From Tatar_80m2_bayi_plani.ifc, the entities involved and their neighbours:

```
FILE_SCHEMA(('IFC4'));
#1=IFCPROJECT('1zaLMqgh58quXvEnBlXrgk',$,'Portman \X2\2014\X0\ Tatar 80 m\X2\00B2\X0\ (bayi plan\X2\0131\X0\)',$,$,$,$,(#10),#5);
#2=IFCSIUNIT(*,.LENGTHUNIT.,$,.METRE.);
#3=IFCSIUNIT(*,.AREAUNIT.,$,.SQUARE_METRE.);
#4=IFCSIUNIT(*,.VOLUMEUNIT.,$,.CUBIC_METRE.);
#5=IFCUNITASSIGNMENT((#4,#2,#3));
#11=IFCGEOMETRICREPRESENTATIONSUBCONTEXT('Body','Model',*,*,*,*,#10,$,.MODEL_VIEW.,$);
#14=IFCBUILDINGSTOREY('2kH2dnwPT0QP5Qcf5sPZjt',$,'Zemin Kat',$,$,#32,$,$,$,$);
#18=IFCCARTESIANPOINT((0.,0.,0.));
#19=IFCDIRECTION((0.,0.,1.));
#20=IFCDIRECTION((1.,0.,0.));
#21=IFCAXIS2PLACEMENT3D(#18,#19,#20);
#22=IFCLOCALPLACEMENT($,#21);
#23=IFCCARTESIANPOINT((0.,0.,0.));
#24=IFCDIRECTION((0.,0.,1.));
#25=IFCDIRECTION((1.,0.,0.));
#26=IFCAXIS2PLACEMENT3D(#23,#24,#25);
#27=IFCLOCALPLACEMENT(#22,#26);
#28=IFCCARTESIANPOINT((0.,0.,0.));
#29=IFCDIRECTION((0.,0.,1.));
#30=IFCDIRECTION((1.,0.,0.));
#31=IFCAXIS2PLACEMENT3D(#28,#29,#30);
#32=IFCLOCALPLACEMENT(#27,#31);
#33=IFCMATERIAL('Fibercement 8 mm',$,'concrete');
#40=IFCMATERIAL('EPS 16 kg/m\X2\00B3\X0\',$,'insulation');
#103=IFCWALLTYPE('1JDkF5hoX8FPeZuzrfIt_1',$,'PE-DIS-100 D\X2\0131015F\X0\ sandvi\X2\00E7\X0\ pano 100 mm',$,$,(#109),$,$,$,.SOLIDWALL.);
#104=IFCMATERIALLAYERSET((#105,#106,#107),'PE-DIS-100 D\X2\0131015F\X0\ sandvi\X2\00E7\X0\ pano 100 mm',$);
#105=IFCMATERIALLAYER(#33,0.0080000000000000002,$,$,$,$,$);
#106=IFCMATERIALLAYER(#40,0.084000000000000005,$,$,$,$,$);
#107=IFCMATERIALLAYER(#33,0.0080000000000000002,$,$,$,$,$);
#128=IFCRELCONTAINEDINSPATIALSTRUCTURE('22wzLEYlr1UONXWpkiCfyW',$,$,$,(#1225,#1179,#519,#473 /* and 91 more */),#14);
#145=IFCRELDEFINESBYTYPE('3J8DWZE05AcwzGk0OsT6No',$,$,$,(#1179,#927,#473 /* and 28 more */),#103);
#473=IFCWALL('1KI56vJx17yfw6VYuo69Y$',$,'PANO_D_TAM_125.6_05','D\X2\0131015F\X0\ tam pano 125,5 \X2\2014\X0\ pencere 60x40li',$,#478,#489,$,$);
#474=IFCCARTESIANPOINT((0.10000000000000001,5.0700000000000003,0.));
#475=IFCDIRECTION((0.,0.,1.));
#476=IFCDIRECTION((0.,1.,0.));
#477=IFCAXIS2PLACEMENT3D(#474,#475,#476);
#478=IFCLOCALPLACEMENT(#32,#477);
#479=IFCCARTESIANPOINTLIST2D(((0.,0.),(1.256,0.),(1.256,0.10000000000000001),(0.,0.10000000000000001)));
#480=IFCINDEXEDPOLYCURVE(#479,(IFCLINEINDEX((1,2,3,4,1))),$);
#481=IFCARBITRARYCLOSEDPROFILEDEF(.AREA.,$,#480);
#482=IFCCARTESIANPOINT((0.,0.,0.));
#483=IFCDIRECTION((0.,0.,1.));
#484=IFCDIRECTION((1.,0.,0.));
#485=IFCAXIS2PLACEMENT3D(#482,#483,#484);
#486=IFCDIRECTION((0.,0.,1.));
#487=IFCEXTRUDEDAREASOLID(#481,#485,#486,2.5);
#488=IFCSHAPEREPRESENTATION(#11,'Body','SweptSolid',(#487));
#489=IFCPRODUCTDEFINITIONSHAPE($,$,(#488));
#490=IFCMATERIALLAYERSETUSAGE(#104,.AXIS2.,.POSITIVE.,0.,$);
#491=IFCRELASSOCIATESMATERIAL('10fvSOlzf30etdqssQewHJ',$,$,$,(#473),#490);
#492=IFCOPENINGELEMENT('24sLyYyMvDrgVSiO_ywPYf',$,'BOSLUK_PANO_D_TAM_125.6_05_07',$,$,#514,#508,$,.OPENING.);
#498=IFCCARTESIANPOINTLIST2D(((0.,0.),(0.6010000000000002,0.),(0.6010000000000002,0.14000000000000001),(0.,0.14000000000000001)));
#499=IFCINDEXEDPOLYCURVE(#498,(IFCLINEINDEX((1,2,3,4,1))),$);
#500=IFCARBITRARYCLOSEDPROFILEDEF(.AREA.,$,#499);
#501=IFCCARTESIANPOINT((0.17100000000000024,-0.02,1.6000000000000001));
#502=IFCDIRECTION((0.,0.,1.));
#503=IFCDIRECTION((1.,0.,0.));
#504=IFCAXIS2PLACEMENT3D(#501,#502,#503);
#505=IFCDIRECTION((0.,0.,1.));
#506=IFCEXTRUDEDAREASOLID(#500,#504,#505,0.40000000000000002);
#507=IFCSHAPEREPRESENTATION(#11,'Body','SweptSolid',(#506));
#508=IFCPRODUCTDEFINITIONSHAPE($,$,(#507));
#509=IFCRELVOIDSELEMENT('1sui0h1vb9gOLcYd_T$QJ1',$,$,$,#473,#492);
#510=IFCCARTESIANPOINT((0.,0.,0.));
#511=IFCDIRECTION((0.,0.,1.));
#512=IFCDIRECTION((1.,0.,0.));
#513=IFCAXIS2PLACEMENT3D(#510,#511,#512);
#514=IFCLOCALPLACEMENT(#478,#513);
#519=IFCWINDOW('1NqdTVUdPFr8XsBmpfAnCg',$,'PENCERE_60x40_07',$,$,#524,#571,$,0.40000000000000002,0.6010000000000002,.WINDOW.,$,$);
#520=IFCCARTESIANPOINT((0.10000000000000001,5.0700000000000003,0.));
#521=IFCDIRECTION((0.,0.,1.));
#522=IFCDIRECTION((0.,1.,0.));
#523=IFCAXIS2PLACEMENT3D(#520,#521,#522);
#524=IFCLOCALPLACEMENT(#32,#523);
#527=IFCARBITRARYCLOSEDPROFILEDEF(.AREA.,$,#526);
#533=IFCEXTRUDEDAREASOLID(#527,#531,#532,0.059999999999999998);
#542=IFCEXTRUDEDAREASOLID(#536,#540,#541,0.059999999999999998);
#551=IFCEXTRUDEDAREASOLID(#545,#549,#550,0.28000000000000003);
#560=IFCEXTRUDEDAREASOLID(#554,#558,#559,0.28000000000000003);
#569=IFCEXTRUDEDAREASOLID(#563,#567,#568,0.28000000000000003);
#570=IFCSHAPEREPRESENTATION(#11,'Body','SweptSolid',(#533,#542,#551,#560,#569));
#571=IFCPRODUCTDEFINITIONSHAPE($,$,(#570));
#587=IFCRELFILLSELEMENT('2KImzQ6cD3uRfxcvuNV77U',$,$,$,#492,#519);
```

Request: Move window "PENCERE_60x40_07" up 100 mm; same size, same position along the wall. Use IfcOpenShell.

```python
import numpy as np
import ifcopenshell
import ifcopenshell.api.geometry
import ifcopenshell.util.placement
import ifcopenshell.util.unit

model = ifcopenshell.open("Tatar_80m2_bayi_plani.ifc")
unit_scale = ifcopenshell.util.unit.calculate_unit_scale(model)

window = model.by_id(519)
opening = window.FillsVoids[0].RelatingOpeningElement
dz = 0.1 / unit_scale

shift = np.array([0.0, 0.0, dz])
# The window is not placed relative to its opening, so move both.
for product in (opening, window):
    matrix = ifcopenshell.util.placement.get_local_placement(product.ObjectPlacement)
    matrix[:3, 3] += shift
    ifcopenshell.api.geometry.edit_object_placement(model, product=product, matrix=matrix, is_si=False)

print(f"moved by {dz * unit_scale:+.3f} m")

model.write("Tatar_80m2_bayi_plani-out.ifc")
```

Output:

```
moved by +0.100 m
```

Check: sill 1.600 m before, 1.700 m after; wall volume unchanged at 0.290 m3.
